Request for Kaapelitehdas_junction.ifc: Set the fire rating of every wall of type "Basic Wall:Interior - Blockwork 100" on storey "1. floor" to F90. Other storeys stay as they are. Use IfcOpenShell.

First a look at what the model holds.

```python
import ifcopenshell
import ifcopenshell.util.element

model = ifcopenshell.open("Kaapelitehdas_junction.ifc")
print(model.schema)
storey = next(s for s in model.by_type("IfcBuildingStorey") if s.Name == "1. floor")
walls = [e for e in ifcopenshell.util.element.get_decomposition(storey) if e.is_a("IfcWall")]
seen = {}
for e in walls:
    element_type = ifcopenshell.util.element.get_type(e)
    key = (element_type.Name if element_type != e and element_type else None, ifcopenshell.util.element.get_pset(e, "Pset_WallCommon", "FireRating"))
    seen[key] = seen.get(key, 0) + 1
for (name, value), count in sorted(seen.items(), key=str):
    print(count, "x", name, "|", value)
```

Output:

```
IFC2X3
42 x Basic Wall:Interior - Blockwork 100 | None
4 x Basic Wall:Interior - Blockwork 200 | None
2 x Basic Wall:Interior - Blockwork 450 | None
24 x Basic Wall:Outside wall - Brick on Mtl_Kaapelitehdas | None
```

```python
import ifcopenshell
import ifcopenshell.api.pset
import ifcopenshell.util.element

model = ifcopenshell.open("Kaapelitehdas_junction.ifc")

storey = next(s for s in model.by_type("IfcBuildingStorey") if s.Name == "1. floor")
walls = [e for e in ifcopenshell.util.element.get_decomposition(storey) if e.is_a("IfcWall")]

count = 0
for e in walls:
    element_type = ifcopenshell.util.element.get_type(e)
    if element_type in (None, e) or element_type.Name != "Basic Wall:Interior - Blockwork 100":
        continue
    # add_pset returns the element's existing set when there is one.
    pset = ifcopenshell.api.pset.add_pset(model, product=e, name="Pset_WallCommon")
    ifcopenshell.api.pset.edit_pset(model, pset=pset, properties={"FireRating": "F90"})
    count += 1

print(count, "walls updated")

model.write("Kaapelitehdas_junction_edited.ifc")
```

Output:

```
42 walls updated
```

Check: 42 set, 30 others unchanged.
